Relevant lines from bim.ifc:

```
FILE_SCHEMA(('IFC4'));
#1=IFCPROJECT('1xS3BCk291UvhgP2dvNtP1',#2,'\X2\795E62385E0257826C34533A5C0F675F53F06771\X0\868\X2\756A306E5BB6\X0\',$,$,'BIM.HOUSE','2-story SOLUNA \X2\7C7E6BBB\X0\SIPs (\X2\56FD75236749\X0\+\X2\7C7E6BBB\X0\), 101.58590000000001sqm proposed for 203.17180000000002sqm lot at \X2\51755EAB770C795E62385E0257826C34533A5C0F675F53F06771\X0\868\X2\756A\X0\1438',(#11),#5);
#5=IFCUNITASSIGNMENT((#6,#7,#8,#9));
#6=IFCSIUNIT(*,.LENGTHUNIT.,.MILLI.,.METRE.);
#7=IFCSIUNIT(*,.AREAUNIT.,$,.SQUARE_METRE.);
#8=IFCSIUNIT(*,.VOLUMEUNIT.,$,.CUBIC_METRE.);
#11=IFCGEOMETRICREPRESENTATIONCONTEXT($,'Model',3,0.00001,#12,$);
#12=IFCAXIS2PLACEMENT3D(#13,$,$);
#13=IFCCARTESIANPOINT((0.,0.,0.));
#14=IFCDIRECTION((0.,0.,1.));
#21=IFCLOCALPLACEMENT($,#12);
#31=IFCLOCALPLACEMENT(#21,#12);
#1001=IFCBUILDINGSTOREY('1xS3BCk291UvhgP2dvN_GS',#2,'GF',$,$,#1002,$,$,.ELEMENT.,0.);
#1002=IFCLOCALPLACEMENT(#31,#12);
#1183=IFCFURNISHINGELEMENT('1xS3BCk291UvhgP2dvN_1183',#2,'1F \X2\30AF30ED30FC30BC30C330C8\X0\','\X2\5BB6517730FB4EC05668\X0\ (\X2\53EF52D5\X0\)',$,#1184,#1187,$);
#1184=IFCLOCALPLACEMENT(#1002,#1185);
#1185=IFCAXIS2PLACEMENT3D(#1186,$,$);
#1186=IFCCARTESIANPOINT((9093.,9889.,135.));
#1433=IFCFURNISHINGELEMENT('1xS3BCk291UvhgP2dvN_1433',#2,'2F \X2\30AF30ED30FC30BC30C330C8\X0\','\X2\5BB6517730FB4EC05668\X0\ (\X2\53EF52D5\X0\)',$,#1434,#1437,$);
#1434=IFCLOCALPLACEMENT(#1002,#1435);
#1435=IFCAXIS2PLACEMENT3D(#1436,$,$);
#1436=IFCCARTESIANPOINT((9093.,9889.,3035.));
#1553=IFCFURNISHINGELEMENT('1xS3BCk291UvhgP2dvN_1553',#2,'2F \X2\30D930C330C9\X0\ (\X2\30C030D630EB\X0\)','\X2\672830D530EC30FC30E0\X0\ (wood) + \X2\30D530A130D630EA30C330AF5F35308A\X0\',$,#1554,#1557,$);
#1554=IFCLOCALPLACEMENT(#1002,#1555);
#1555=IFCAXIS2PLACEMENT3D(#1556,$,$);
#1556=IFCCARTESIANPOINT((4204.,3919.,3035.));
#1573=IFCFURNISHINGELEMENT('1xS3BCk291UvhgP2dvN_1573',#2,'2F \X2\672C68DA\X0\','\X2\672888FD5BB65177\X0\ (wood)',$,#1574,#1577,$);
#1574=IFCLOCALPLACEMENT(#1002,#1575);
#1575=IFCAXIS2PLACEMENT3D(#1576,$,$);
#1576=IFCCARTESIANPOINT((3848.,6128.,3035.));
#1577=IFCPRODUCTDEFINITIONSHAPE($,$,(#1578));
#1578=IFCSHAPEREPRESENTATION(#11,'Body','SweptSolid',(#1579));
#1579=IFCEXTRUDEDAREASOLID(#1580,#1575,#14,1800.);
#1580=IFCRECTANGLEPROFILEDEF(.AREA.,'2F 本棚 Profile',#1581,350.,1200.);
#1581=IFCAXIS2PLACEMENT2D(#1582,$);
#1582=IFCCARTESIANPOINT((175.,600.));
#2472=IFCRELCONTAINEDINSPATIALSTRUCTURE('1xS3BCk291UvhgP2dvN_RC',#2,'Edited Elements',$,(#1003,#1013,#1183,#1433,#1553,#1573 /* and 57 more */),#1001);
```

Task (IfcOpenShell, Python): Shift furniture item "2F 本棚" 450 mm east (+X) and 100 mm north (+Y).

```python
import ifcopenshell
import ifcopenshell.api.geometry
import ifcopenshell.util.placement
import ifcopenshell.util.unit

model = ifcopenshell.open("bim.ifc")
unit_scale = ifcopenshell.util.unit.calculate_unit_scale(model)

item = model.by_guid("1xS3BCk291UvhgP2dvN_1573")
matrix = ifcopenshell.util.placement.get_local_placement(item.ObjectPlacement)
matrix[0, 3] += 0.45 / unit_scale
matrix[1, 3] += 0.1 / unit_scale
ifcopenshell.api.geometry.edit_object_placement(model, product=item, matrix=matrix, is_si=False)

print(ifcopenshell.util.placement.get_local_placement(item.ObjectPlacement).round(3) + 0.0)

model.write("bim_updated.ifc")
```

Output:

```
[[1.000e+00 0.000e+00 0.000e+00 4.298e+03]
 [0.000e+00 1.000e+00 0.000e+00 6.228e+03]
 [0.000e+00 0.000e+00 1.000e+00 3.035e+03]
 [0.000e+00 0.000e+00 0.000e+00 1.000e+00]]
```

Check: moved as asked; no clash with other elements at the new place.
